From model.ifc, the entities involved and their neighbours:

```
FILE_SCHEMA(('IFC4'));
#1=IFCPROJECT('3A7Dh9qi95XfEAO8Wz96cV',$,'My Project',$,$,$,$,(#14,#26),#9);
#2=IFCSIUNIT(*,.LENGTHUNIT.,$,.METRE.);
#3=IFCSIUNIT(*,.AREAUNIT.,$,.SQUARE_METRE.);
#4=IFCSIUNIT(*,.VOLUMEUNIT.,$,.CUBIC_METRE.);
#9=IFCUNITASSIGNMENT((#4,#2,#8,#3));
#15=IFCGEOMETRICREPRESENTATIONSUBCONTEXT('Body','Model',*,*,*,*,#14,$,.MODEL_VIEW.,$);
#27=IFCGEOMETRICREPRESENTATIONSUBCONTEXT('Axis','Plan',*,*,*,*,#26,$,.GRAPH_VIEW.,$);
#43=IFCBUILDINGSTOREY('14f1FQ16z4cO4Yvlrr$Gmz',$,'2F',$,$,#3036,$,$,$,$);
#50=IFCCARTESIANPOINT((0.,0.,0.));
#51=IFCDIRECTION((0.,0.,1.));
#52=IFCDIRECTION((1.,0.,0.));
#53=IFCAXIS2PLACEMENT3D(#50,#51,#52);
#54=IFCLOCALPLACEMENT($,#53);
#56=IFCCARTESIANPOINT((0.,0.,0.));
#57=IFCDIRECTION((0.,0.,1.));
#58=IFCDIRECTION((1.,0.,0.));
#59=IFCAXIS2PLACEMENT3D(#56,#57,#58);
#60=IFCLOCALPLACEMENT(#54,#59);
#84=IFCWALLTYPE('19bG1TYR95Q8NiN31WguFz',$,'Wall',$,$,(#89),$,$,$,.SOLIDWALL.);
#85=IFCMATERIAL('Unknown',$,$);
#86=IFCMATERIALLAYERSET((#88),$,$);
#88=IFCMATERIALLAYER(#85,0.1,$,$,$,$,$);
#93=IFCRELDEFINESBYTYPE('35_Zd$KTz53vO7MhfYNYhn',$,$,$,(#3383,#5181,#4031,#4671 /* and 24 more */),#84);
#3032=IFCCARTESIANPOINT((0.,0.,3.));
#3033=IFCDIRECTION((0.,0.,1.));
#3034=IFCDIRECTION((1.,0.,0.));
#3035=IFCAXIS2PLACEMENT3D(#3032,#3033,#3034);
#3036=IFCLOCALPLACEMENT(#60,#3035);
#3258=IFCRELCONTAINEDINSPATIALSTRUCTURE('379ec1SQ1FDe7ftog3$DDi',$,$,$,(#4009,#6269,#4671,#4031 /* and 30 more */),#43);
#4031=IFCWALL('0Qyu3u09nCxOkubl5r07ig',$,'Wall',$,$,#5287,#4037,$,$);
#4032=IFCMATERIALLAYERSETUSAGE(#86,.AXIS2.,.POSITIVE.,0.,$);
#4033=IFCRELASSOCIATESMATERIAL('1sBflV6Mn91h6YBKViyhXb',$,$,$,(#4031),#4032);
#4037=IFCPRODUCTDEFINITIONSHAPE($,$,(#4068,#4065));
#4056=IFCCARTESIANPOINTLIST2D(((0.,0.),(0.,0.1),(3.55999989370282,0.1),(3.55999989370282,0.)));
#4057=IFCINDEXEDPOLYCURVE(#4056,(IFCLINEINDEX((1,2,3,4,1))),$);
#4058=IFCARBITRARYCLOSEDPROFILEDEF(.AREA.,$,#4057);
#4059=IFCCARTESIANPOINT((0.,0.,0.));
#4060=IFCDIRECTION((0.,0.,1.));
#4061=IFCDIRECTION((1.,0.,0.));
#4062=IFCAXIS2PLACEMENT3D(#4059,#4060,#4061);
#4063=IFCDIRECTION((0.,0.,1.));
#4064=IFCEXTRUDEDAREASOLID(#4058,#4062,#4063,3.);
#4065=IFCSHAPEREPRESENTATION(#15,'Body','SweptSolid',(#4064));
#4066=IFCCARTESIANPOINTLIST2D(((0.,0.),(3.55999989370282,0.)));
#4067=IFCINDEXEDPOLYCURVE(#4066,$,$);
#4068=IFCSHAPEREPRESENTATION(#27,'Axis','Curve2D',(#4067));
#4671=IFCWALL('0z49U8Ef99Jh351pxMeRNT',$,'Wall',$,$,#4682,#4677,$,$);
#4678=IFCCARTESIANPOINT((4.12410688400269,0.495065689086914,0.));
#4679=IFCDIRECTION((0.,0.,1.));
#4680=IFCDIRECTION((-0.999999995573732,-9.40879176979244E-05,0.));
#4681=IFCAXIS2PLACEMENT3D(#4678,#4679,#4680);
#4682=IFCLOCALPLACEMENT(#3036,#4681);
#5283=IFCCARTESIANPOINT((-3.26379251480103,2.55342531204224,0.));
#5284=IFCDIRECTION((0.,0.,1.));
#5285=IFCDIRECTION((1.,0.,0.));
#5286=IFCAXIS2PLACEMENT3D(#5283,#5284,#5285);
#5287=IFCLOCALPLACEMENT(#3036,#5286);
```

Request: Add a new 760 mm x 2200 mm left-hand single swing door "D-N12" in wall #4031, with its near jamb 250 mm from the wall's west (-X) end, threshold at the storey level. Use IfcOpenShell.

```python
import numpy as np
import ifcopenshell
import ifcopenshell.api.feature
import ifcopenshell.api.geometry
import ifcopenshell.api.root
import ifcopenshell.api.spatial
import ifcopenshell.geom
import ifcopenshell.util.element
import ifcopenshell.util.placement
import ifcopenshell.util.representation
import ifcopenshell.util.shape
import ifcopenshell.util.unit

model = ifcopenshell.open("model.ifc")
unit_scale = ifcopenshell.util.unit.calculate_unit_scale(model)
settings = ifcopenshell.geom.settings()


def volume(element):
    """Net volume in cubic metres, openings subtracted."""
    shape = ifcopenshell.geom.create_shape(settings, element)
    return ifcopenshell.util.shape.get_volume(shape.geometry)


wall = model.by_guid("0Qyu3u09nCxOkubl5r07ig")
storey = ifcopenshell.util.element.get_container(wall, ifc_class="IfcBuildingStorey")
context = ifcopenshell.util.representation.get_context(model, "Model", "Body", "MODEL_VIEW")
before = volume(wall)

width, height, from_end, sill = 0.76, 2.2, 0.25, 0.0  # metres

# The wall runs along its own X axis, and the end named is its -X end.
wall_shape = ifcopenshell.geom.create_shape(settings, wall)
x, y, z = ifcopenshell.util.shape.get_vertices(wall_shape.geometry).T
start = x.min() + from_end
face, thickness = float(y.min()), float(y.max() - y.min())
wall_matrix = ifcopenshell.util.placement.get_local_placement(wall.ObjectPlacement)
level = ifcopenshell.util.placement.get_local_placement(storey.ObjectPlacement)[2, 3]


def in_wall(x, y):
    """Placement at x, y metres in the wall's axes, at sill height."""
    matrix = wall_matrix.copy()
    matrix[:, 3] = wall_matrix @ np.array([x / unit_scale, y / unit_scale, 0.0, 1.0])
    matrix[2, 3] = level + sill / unit_scale
    return matrix


# Opening: a box that overshoots both wall faces by 50 mm.
opening = ifcopenshell.api.root.create_entity(model, ifc_class="IfcOpeningElement", predefined_type="OPENING")
box = ifcopenshell.api.geometry.add_wall_representation(
    model, context=context, length=width, height=height, thickness=thickness + 0.1
)
ifcopenshell.api.geometry.assign_representation(model, product=opening, representation=box)
ifcopenshell.api.geometry.edit_object_placement(model, product=opening, matrix=in_wall(start, face - 0.05), is_si=False)
ifcopenshell.api.feature.add_feature(model, feature=opening, element=wall)

door = ifcopenshell.api.root.create_entity(model, ifc_class="IfcDoor", name="D-N12", predefined_type="DOOR")
door.OverallWidth, door.OverallHeight = width / unit_scale, height / unit_scale
door.OperationType = "SINGLE_SWING_LEFT"
body = ifcopenshell.api.geometry.add_door_representation(
    model,
    context=context,
    overall_width=door.OverallWidth,
    overall_height=door.OverallHeight,
    operation_type="SINGLE_SWING_LEFT",
    lining_properties={"LiningDepth": thickness / unit_scale, "ThresholdDepth": thickness / unit_scale},
)
ifcopenshell.api.geometry.assign_representation(model, product=door, representation=body)
ifcopenshell.api.spatial.assign_container(model, products=[door], relating_structure=storey)
ifcopenshell.api.feature.add_filling(model, opening=opening, element=door)

# The lining spans the wall, so the door starts at the wall face.
ifcopenshell.api.geometry.edit_object_placement(model, product=door, matrix=in_wall(start, face), is_si=False)

after = volume(wall)

print(f"wall volume {before:.3f} -> {after:.3f} m3")

model.write("model-out.ifc")
```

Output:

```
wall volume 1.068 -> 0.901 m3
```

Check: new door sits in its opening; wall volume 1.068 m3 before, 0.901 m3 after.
